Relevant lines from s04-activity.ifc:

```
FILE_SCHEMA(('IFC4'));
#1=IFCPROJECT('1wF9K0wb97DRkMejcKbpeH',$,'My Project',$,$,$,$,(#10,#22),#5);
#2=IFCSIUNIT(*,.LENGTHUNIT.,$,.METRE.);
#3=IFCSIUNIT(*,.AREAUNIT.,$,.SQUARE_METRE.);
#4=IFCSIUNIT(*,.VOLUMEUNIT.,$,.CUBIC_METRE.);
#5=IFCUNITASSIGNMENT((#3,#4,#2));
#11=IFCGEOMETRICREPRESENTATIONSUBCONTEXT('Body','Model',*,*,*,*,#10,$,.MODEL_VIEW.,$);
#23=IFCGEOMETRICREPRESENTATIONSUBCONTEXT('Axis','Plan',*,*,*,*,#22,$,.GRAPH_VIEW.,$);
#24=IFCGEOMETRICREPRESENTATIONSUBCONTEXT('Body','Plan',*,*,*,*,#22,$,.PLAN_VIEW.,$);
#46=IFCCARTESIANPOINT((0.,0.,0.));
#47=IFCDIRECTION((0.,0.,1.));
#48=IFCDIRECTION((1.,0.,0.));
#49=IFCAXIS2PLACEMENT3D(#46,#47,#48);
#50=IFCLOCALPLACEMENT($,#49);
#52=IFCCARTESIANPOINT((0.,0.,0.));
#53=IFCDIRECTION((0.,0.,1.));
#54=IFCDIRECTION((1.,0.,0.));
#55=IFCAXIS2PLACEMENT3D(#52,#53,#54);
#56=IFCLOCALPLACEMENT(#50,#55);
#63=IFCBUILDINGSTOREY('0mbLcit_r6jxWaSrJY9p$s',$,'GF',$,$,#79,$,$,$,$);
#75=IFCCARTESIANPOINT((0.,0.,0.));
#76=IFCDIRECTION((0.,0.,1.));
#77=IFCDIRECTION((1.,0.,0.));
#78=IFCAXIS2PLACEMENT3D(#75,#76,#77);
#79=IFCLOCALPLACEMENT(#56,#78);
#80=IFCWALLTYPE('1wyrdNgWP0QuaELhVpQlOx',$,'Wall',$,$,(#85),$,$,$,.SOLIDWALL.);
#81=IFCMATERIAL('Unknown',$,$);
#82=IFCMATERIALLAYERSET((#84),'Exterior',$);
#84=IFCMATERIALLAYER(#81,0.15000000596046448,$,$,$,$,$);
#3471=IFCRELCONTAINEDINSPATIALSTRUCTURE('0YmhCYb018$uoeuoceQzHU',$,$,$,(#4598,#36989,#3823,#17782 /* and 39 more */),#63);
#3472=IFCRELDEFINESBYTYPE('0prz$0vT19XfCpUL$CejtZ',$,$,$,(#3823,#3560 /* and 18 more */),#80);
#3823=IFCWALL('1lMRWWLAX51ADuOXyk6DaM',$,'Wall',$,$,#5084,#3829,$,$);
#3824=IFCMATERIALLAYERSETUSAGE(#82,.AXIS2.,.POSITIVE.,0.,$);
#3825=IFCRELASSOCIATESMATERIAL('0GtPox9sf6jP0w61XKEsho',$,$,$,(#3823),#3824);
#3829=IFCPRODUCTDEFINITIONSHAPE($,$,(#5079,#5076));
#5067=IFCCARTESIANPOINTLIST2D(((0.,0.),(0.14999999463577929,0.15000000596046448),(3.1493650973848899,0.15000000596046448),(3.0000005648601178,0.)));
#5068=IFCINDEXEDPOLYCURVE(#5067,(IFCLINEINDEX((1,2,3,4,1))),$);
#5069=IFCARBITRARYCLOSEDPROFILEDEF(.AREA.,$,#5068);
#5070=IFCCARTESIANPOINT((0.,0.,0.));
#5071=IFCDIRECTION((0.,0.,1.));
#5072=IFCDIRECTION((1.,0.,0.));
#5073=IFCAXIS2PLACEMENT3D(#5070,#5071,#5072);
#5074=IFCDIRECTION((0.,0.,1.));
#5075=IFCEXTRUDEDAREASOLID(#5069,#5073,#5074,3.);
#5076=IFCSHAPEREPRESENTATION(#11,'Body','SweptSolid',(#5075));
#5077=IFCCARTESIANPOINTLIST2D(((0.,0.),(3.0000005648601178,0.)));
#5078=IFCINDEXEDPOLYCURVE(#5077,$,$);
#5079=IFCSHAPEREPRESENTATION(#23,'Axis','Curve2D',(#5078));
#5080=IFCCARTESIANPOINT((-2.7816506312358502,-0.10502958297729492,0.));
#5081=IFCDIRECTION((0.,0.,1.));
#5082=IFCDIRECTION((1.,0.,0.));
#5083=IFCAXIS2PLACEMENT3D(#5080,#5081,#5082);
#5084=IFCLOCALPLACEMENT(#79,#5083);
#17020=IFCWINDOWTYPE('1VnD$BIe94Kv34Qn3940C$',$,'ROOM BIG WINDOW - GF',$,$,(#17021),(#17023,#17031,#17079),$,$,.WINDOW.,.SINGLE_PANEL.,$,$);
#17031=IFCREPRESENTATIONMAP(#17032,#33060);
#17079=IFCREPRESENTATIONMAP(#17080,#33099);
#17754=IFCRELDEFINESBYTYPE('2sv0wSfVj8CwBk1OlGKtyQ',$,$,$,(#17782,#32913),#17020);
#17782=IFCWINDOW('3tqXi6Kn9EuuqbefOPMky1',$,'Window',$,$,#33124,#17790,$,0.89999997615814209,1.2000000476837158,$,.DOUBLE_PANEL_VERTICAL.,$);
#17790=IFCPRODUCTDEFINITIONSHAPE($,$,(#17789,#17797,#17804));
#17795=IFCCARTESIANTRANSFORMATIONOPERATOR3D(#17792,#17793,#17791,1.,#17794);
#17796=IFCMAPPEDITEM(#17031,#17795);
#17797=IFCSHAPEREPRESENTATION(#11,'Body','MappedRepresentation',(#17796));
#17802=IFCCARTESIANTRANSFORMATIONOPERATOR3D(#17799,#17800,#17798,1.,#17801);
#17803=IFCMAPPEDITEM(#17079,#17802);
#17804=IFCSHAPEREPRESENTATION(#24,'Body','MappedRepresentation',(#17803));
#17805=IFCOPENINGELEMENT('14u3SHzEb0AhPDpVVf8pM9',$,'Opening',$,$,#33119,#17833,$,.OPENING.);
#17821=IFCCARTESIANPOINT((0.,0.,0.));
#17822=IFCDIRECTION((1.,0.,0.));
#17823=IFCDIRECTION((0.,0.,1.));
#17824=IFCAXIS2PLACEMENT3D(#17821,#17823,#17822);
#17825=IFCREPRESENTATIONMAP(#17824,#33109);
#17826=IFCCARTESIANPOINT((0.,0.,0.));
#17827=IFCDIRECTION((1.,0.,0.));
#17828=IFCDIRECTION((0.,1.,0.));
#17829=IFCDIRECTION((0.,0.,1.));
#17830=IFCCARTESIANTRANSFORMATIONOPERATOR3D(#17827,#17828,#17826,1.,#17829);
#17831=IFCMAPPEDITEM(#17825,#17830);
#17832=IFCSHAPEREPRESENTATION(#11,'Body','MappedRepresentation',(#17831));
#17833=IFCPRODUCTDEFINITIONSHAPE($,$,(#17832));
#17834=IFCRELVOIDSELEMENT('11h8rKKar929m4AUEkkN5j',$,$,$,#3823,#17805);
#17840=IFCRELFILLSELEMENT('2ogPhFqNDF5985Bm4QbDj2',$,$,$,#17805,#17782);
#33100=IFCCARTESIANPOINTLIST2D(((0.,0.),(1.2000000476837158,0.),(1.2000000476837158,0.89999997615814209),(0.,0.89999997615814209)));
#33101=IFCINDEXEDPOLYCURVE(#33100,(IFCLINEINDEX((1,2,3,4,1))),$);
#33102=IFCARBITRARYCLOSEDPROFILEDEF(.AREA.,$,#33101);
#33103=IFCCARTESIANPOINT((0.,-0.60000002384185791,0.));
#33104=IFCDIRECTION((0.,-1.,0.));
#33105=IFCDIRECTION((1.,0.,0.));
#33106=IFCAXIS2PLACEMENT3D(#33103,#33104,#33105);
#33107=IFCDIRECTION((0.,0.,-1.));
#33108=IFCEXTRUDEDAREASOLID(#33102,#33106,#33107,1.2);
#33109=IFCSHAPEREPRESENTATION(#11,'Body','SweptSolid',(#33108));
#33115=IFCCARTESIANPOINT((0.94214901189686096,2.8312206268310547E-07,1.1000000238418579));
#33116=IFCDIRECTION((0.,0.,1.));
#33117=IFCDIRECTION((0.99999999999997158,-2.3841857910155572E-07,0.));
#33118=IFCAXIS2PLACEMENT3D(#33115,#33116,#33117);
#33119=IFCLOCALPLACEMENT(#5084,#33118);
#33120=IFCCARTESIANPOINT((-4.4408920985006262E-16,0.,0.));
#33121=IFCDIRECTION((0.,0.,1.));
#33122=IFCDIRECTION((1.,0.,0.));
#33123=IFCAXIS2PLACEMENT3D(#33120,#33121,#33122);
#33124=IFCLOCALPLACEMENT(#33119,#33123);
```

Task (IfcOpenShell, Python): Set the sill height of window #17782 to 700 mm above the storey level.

```python
import numpy as np
import ifcopenshell
import ifcopenshell.api.geometry
import ifcopenshell.geom
import ifcopenshell.util.element
import ifcopenshell.util.placement
import ifcopenshell.util.shape
import ifcopenshell.util.unit

model = ifcopenshell.open("s04-activity.ifc")
unit_scale = ifcopenshell.util.unit.calculate_unit_scale(model)

window = model.by_guid("3tqXi6Kn9EuuqbefOPMky1")
opening = window.FillsVoids[0].RelatingOpeningElement
storey = ifcopenshell.util.element.get_container(window, ifc_class="IfcBuildingStorey")
level = ifcopenshell.util.placement.get_local_placement(storey.ObjectPlacement)[2, 3]

# The opening's origin need not be at the sill, so measure its lowest point.
shape = ifcopenshell.geom.create_shape(ifcopenshell.geom.settings(), opening)
bottom = ifcopenshell.util.shape.get_shape_bottom_elevation(shape, shape.geometry) / unit_scale
dz = level + 0.7 - bottom

shift = np.array([0.0, 0.0, dz])
# The window is placed relative to its opening, so it follows when the opening moves.
matrix = ifcopenshell.util.placement.get_local_placement(opening.ObjectPlacement)
matrix[:3, 3] += shift
ifcopenshell.api.geometry.edit_object_placement(
    model, product=opening, matrix=matrix, is_si=False, should_transform_children=True
)

print(f"moved by {dz * unit_scale:+.3f} m")

model.write("s04-activity_v2.ifc")
```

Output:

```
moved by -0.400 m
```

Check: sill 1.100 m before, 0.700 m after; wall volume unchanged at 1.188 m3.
